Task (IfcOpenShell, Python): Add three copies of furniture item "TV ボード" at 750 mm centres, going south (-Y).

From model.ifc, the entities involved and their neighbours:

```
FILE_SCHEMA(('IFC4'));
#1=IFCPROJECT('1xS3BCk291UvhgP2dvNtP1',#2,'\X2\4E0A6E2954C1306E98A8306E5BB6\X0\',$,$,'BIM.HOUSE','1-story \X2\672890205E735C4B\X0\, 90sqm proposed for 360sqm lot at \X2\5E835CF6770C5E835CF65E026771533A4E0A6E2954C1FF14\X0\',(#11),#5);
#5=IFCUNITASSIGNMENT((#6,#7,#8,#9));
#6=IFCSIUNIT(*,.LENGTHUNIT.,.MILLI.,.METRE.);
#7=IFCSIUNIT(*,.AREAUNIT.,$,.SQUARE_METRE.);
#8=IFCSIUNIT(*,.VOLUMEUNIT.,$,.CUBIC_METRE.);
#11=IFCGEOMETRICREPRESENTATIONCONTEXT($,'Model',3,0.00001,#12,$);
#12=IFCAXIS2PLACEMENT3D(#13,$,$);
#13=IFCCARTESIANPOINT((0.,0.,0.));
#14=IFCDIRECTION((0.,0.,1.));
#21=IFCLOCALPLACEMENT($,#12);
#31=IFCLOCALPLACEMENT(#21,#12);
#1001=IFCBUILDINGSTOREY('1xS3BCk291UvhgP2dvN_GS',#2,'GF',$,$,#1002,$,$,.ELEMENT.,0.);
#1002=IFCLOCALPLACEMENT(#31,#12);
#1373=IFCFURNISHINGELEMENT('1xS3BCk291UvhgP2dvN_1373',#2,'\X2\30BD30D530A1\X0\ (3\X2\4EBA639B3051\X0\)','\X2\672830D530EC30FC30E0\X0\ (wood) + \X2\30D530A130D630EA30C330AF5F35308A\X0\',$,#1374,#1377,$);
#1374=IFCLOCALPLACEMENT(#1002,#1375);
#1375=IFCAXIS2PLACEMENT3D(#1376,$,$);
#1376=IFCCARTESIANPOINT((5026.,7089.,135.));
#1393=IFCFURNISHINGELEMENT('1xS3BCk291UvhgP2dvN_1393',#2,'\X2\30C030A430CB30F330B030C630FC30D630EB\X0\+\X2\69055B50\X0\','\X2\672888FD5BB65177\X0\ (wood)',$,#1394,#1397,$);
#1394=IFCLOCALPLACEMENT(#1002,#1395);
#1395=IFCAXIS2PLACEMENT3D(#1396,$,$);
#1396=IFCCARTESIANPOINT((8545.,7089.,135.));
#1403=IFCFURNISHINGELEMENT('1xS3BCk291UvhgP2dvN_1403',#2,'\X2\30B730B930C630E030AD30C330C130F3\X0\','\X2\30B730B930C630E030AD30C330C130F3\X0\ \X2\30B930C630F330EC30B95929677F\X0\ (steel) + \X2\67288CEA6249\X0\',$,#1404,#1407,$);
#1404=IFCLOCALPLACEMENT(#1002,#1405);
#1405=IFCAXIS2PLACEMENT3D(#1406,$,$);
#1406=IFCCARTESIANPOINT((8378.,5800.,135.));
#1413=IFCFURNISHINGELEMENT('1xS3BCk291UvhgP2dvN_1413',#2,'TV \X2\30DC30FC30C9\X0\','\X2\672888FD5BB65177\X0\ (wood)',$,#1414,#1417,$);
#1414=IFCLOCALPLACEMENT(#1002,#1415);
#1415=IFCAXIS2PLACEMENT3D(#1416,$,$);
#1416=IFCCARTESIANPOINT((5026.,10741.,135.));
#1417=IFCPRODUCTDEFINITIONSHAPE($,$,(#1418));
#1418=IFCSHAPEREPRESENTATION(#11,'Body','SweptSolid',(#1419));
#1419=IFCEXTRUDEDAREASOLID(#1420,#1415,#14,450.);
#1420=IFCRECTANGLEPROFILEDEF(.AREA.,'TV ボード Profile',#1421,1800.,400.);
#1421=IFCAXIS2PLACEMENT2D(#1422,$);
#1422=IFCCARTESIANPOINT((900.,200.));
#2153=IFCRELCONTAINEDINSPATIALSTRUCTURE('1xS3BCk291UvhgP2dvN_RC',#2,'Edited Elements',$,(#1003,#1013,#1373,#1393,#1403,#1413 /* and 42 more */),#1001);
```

```python
import numpy as np
import ifcopenshell
import ifcopenshell.api.geometry
import ifcopenshell.api.root
import ifcopenshell.util.element
import ifcopenshell.util.placement
import ifcopenshell.util.unit

model = ifcopenshell.open("model.ifc")
unit_scale = ifcopenshell.util.unit.calculate_unit_scale(model)


def reuse_history(source, copy):
    """copy_class also copies each property set's owner history, people and application; keep the originals."""
    for rel in copy.IsDefinedBy:
        if rel.is_a("IfcRelDefinesByProperties") and (history := rel.RelatingPropertyDefinition.OwnerHistory):
            rel.RelatingPropertyDefinition.OwnerHistory = source.OwnerHistory
            ifcopenshell.util.element.remove_deep2(model, history)


source = model.by_guid("1xS3BCk291UvhgP2dvN_1413")
base = ifcopenshell.util.placement.get_local_placement(source.ObjectPlacement)
step = np.array([0.0, -1.0, 0.0]) * 0.75 / unit_scale

for i in range(1, 4):
    copy = ifcopenshell.api.root.copy_class(model, product=source)
    copy.Representation = ifcopenshell.util.element.copy_deep(
        model, source.Representation, exclude=["IfcGeometricRepresentationContext", "IfcRepresentationMap"]
    )
    reuse_history(source, copy)
    matrix = base.copy()
    matrix[:3, 3] += i * step
    print("added at", matrix[:3, 3].round(3) + 0.0)
    ifcopenshell.api.geometry.edit_object_placement(model, product=copy, matrix=matrix, is_si=False)

model.write("model_rev.ifc")
```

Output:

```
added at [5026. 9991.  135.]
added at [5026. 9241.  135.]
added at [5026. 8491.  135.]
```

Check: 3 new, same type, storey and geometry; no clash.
